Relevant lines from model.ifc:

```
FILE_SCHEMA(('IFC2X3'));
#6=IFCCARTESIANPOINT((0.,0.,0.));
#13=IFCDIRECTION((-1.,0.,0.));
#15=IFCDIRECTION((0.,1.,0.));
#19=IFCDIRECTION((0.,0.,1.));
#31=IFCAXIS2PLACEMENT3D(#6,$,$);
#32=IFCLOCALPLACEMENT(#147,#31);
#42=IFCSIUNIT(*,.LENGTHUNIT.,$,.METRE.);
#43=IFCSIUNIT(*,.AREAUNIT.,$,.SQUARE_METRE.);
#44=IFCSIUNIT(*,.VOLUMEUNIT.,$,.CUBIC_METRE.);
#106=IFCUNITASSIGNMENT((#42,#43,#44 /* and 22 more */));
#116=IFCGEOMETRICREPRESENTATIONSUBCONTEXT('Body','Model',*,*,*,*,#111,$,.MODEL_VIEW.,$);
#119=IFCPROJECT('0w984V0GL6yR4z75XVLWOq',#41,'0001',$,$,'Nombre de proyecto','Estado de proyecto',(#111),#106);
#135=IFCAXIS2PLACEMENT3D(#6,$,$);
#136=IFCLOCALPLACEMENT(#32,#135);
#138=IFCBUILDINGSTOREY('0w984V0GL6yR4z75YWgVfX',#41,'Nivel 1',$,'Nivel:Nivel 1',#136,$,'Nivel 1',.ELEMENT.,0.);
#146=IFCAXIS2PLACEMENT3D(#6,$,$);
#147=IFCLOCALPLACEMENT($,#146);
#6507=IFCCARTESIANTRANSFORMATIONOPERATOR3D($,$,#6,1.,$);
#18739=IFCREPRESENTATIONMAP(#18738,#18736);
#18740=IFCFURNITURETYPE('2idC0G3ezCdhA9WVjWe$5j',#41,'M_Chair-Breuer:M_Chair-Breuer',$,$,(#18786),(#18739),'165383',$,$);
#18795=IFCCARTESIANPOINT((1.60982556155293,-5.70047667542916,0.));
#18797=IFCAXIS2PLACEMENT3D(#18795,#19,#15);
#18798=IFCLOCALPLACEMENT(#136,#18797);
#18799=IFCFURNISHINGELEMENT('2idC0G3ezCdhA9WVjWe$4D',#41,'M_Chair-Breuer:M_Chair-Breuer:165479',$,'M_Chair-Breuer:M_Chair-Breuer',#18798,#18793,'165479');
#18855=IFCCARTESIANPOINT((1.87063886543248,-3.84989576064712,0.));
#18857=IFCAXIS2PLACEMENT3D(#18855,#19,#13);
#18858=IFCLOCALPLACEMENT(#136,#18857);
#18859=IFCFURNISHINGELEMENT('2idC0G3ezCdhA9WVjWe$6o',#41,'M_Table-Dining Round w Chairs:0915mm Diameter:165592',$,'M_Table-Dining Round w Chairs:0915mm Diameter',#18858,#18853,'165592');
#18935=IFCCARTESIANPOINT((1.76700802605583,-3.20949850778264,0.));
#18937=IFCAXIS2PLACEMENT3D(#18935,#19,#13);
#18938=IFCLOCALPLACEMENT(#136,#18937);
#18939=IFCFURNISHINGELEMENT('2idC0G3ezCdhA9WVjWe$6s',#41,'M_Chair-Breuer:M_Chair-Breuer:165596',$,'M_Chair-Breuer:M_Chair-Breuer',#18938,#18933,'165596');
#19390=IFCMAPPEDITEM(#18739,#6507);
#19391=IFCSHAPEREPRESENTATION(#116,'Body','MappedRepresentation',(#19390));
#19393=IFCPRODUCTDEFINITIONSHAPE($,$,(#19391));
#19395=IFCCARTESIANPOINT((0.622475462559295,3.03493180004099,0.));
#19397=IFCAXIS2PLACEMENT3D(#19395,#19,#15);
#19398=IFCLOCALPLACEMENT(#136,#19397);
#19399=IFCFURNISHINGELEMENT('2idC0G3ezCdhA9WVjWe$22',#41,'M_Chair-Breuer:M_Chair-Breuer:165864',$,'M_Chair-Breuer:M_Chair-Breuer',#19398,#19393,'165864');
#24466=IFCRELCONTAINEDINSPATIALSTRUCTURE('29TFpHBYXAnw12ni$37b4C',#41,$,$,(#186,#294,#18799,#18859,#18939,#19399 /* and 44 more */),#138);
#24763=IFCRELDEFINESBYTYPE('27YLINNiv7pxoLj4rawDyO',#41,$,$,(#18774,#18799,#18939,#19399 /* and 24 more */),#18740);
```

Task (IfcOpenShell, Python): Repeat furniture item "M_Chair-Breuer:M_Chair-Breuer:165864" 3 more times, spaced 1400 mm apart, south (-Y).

```python
import numpy as np
import ifcopenshell
import ifcopenshell.api.geometry
import ifcopenshell.api.root
import ifcopenshell.util.element
import ifcopenshell.util.placement
import ifcopenshell.util.unit

model = ifcopenshell.open("model.ifc")
unit_scale = ifcopenshell.util.unit.calculate_unit_scale(model)


def reuse_history(source, copy):
    """copy_class also copies each property set's owner history, people and application; keep the originals."""
    for rel in copy.IsDefinedBy:
        if rel.is_a("IfcRelDefinesByProperties") and (history := rel.RelatingPropertyDefinition.OwnerHistory):
            rel.RelatingPropertyDefinition.OwnerHistory = source.OwnerHistory
            ifcopenshell.util.element.remove_deep2(model, history)


source = model.by_id(19399)
base = ifcopenshell.util.placement.get_local_placement(source.ObjectPlacement)
step = np.array([0.0, -1.0, 0.0]) * 1.4 / unit_scale

for i in range(1, 4):
    copy = ifcopenshell.api.root.copy_class(model, product=source)
    copy.Representation = ifcopenshell.util.element.copy_deep(
        model, source.Representation, exclude=["IfcGeometricRepresentationContext", "IfcRepresentationMap"]
    )
    copy.Name = "M_Chair-Breuer:M_Chair-Breuer"
    copy.Tag = None
    reuse_history(source, copy)
    matrix = base.copy()
    matrix[:3, 3] += i * step
    print("added at", matrix[:3, 3].round(3) + 0.0)
    ifcopenshell.api.geometry.edit_object_placement(model, product=copy, matrix=matrix, is_si=False)

model.write("model-out.ifc")
```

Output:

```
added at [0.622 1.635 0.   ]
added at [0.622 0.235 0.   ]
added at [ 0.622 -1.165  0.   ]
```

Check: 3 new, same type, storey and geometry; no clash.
